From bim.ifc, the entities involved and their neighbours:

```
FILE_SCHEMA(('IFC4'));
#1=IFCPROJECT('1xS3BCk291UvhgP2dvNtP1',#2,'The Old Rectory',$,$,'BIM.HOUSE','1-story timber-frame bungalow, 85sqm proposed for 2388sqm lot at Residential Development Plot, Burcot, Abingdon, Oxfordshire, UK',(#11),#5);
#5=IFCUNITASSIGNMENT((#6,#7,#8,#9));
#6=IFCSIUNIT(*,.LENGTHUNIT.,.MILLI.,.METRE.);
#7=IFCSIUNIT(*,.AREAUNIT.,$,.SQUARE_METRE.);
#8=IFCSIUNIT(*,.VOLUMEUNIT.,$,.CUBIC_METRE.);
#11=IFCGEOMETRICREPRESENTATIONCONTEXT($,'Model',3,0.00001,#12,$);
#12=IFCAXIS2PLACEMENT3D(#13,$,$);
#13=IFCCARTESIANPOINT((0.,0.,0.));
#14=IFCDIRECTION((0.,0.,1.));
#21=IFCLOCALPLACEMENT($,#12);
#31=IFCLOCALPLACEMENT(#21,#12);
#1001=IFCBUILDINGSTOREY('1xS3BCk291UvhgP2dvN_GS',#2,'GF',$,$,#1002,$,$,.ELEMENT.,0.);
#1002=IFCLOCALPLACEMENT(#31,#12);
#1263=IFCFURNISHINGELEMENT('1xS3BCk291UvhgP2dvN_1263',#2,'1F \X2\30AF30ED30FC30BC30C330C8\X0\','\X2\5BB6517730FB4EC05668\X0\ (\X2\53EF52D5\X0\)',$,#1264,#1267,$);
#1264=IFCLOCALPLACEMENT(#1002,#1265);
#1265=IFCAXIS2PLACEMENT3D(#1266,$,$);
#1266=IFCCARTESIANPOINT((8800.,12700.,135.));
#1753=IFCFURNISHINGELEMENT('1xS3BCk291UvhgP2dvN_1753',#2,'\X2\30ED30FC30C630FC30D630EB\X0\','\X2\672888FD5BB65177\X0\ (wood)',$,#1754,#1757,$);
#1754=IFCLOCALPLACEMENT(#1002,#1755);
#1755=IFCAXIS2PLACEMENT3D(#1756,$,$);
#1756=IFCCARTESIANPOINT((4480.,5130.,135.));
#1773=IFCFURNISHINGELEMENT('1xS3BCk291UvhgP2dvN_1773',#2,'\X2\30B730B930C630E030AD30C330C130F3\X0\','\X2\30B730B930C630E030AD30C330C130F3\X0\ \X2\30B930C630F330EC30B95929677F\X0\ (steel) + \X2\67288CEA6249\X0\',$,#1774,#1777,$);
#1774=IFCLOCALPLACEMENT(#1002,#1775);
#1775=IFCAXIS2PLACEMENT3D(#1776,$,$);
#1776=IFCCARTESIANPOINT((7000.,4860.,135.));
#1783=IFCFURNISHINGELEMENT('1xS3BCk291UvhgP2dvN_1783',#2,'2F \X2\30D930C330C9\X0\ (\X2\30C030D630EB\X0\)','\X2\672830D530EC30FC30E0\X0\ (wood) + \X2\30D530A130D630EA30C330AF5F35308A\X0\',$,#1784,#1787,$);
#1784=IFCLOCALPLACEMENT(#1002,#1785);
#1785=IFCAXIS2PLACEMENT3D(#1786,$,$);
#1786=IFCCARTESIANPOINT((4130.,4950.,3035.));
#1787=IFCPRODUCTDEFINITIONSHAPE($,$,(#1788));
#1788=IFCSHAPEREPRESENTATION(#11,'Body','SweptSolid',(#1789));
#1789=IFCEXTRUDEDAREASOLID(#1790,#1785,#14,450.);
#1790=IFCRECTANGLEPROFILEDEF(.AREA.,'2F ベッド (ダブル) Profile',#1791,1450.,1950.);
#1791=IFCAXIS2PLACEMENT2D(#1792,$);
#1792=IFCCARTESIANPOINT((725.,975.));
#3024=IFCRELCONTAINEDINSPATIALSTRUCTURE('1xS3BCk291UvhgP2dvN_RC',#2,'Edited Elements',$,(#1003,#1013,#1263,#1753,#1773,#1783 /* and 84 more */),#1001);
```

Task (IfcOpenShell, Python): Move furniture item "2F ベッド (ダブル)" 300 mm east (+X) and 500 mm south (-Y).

```python
import ifcopenshell
import ifcopenshell.api.geometry
import ifcopenshell.util.placement
import ifcopenshell.util.unit

model = ifcopenshell.open("bim.ifc")
unit_scale = ifcopenshell.util.unit.calculate_unit_scale(model)

item = model.by_guid("1xS3BCk291UvhgP2dvN_1783")
matrix = ifcopenshell.util.placement.get_local_placement(item.ObjectPlacement)
matrix[0, 3] += 0.3 / unit_scale
matrix[1, 3] -= 0.5 / unit_scale
ifcopenshell.api.geometry.edit_object_placement(model, product=item, matrix=matrix, is_si=False)

print(ifcopenshell.util.placement.get_local_placement(item.ObjectPlacement).round(3) + 0.0)

model.write("bim-out.ifc")
```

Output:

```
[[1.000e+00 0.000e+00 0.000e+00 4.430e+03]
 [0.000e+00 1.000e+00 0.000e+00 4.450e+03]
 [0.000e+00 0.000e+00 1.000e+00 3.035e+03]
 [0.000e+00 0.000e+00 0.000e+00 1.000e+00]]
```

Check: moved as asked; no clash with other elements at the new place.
